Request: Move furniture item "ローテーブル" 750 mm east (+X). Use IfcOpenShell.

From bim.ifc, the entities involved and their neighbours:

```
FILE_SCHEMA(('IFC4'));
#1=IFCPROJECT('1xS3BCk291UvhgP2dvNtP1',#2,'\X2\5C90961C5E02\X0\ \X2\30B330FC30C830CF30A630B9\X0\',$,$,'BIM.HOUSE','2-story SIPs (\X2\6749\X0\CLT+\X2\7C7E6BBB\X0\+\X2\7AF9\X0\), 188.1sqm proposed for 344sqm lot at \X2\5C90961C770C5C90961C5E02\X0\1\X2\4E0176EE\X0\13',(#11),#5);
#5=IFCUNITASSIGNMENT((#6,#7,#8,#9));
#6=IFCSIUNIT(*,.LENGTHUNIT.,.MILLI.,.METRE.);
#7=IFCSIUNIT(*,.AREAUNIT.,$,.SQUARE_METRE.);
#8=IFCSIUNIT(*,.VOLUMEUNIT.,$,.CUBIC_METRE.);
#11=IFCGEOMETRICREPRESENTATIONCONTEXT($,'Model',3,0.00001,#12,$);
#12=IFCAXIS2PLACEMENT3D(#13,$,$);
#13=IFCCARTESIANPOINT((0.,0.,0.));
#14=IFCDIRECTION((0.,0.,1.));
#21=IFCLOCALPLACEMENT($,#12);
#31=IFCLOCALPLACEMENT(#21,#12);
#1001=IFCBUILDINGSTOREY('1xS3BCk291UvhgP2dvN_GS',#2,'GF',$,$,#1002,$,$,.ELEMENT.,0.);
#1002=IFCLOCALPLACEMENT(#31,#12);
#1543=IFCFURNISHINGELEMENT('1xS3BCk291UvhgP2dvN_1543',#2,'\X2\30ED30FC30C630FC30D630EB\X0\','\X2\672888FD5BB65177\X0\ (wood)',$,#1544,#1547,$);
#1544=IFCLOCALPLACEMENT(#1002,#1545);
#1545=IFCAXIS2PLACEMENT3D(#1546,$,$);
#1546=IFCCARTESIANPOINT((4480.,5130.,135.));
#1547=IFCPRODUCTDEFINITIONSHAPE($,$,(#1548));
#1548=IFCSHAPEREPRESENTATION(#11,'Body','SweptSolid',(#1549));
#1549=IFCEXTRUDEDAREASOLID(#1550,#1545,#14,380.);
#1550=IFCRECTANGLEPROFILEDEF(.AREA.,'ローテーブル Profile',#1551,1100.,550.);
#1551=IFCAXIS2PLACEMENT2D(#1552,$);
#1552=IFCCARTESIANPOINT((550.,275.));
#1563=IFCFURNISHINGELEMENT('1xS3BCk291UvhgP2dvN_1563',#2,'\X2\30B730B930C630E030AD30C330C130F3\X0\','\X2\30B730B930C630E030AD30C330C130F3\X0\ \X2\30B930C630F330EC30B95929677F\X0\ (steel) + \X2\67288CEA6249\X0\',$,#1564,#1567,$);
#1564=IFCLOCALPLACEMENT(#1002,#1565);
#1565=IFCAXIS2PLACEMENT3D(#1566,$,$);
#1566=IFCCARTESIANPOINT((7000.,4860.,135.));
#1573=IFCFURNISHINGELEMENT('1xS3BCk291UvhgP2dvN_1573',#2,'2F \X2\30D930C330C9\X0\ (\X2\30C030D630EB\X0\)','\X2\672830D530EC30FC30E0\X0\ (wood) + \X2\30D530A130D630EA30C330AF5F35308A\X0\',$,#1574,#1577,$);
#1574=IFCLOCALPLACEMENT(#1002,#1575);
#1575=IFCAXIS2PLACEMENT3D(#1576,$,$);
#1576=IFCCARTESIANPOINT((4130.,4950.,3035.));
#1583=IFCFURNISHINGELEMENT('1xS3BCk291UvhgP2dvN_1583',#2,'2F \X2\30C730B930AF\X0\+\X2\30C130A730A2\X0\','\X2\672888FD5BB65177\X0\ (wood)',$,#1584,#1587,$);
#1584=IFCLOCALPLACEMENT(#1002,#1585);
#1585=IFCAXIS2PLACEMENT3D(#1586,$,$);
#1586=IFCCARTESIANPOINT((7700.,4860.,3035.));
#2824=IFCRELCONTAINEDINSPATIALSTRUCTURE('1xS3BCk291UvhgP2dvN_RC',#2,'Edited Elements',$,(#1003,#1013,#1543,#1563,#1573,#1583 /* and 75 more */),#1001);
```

```python
import ifcopenshell
import ifcopenshell.api.geometry
import ifcopenshell.util.placement
import ifcopenshell.util.unit

model = ifcopenshell.open("bim.ifc")
unit_scale = ifcopenshell.util.unit.calculate_unit_scale(model)

item = model.by_id(1543)
matrix = ifcopenshell.util.placement.get_local_placement(item.ObjectPlacement)
matrix[0, 3] += 0.75 / unit_scale
ifcopenshell.api.geometry.edit_object_placement(model, product=item, matrix=matrix, is_si=False)

print(ifcopenshell.util.placement.get_local_placement(item.ObjectPlacement).round(3) + 0.0)

model.write("bim-out.ifc")
```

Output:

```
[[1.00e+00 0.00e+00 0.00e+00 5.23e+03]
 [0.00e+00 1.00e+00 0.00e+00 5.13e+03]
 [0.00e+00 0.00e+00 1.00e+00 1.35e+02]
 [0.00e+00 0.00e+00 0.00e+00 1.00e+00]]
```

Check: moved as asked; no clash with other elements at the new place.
